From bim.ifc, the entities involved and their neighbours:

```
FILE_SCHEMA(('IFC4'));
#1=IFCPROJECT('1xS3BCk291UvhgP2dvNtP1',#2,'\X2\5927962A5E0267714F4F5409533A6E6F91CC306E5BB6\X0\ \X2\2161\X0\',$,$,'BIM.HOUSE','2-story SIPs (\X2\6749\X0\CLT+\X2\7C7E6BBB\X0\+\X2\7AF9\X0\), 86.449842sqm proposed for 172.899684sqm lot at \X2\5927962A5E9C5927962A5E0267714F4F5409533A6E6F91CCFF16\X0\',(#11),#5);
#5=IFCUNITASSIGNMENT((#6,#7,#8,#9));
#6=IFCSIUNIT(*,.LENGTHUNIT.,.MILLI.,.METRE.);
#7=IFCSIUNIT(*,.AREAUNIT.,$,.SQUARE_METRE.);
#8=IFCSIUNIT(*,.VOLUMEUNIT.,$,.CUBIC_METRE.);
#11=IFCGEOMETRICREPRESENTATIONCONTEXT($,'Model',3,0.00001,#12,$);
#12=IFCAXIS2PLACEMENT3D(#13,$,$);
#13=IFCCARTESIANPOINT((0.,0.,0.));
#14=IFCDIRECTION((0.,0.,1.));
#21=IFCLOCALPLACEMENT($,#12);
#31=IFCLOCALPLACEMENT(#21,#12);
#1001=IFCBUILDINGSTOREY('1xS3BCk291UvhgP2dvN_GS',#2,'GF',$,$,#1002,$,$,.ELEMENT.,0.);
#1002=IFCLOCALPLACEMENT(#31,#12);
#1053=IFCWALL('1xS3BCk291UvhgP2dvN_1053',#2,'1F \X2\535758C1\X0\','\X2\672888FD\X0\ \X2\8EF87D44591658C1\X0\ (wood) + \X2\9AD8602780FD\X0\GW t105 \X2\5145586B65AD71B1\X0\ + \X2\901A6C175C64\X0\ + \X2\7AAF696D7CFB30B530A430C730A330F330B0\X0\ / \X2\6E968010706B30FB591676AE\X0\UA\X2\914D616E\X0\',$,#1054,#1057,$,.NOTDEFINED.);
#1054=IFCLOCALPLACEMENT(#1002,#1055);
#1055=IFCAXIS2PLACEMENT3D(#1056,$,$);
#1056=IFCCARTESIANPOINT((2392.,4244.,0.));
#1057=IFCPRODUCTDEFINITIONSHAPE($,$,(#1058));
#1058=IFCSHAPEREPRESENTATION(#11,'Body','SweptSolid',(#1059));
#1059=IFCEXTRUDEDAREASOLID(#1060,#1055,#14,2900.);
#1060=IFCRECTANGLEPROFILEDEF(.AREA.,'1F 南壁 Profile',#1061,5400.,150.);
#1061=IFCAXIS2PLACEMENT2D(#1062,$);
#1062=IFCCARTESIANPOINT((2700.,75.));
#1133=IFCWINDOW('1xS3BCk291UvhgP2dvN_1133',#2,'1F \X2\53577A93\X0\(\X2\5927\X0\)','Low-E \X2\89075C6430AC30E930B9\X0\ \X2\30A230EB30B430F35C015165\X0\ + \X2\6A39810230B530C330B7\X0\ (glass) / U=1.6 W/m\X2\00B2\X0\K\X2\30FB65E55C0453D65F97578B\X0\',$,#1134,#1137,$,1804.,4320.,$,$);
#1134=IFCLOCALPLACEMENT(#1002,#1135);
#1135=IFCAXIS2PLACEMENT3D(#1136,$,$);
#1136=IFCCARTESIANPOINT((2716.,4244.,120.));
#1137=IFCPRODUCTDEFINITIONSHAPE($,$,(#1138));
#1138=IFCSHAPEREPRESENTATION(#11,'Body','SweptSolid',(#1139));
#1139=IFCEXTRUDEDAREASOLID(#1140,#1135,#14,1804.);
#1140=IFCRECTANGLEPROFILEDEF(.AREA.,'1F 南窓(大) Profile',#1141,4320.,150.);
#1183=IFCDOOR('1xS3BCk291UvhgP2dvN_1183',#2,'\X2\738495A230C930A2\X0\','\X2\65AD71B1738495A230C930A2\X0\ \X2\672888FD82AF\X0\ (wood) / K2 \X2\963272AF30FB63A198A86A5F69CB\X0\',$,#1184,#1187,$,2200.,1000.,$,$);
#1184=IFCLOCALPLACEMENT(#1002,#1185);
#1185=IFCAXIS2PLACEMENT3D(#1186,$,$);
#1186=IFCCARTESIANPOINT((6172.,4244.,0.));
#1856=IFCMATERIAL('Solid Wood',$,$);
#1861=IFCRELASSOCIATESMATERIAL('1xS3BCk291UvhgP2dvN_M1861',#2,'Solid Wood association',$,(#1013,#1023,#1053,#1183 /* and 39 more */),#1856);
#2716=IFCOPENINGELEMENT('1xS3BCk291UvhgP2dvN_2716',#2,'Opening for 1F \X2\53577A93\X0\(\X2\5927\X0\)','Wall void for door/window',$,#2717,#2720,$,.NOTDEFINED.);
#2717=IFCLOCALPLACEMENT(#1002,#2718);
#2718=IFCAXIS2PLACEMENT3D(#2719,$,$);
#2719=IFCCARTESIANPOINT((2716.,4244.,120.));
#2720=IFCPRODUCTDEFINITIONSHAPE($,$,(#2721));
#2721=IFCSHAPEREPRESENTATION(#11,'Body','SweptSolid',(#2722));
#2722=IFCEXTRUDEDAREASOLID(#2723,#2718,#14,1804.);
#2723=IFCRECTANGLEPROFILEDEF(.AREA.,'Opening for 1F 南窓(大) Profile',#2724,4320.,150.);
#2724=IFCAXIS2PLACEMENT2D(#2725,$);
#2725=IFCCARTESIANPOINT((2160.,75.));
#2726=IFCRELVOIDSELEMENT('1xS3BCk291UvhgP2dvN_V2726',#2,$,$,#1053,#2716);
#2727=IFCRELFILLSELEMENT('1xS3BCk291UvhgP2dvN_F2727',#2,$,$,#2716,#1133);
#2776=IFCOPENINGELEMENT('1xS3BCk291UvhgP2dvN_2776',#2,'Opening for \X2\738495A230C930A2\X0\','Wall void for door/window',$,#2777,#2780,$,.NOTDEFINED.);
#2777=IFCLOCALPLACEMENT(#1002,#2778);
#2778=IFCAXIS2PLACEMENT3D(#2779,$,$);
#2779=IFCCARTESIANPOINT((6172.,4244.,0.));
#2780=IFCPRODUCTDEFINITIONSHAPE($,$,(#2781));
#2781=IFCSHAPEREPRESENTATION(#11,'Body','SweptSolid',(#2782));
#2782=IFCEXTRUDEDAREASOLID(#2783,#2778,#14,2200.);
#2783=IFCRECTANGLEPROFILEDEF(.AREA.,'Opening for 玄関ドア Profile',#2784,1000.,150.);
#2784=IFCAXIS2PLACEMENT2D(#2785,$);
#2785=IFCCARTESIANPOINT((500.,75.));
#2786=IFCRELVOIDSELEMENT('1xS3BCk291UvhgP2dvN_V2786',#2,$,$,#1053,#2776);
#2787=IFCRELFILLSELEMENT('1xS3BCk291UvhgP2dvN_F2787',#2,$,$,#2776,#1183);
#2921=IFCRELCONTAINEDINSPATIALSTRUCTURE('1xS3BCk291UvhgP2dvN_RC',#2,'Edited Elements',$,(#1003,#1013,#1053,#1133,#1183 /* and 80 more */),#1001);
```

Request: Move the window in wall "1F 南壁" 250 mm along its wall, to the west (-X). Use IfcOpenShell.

```python
import ifcopenshell
import ifcopenshell.api.geometry
import ifcopenshell.util.placement
import ifcopenshell.util.unit

model = ifcopenshell.open("bim.ifc")
unit_scale = ifcopenshell.util.unit.calculate_unit_scale(model)

window = model.by_guid("1xS3BCk291UvhgP2dvN_1133")
opening = window.FillsVoids[0].RelatingOpeningElement
wall = opening.VoidsElements[0].RelatingBuildingElement

wall_matrix = ifcopenshell.util.placement.get_local_placement(wall.ObjectPlacement)
shift = wall_matrix[:3, 0] * -0.25 / unit_scale
before = ifcopenshell.util.placement.get_local_placement(window.ObjectPlacement)[:3, 3].copy()

# The window is not placed relative to its opening, so move both.
for product in (opening, window):
    matrix = ifcopenshell.util.placement.get_local_placement(product.ObjectPlacement)
    matrix[:3, 3] += shift
    ifcopenshell.api.geometry.edit_object_placement(model, product=product, matrix=matrix, is_si=False)

after = ifcopenshell.util.placement.get_local_placement(window.ObjectPlacement)[:3, 3]
print("window moved by", (after - before).round(3) + 0.0)

model.write("bim_edited.ifc")
```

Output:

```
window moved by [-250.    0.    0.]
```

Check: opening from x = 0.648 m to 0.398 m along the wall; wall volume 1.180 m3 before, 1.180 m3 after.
